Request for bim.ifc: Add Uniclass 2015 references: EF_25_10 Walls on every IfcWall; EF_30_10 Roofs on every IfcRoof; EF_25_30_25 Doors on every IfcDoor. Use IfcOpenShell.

First a look at what the model holds.

```python
import ifcopenshell

model = ifcopenshell.open("bim.ifc")
print(model.schema)
print("classifications:", [c.Name for c in model.by_type("IfcClassification")])
for ifc_class in ("IfcDoor", "IfcRoof", "IfcStair", "IfcWall", "IfcWindow"):
    print(ifc_class, len(model.by_type(ifc_class)))
```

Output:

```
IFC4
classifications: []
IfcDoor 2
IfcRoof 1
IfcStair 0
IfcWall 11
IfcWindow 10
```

```python
import ifcopenshell
import ifcopenshell.api.classification

model = ifcopenshell.open("bim.ifc")

system = ifcopenshell.api.classification.add_classification(model, classification="Uniclass 2015")

codes = {
    "IfcWall": ("EF_25_10", "Walls"),
    "IfcRoof": ("EF_30_10", "Roofs"),
    "IfcDoor": ("EF_25_30_25", "Doors"),
}
for ifc_class, (code, name) in codes.items():
    products = model.by_type(ifc_class)
    ifcopenshell.api.classification.add_reference(
        model, products=products, classification=system, identification=code, name=name
    )
    print(code, len(products))

model.write("bim_updated.ifc")
```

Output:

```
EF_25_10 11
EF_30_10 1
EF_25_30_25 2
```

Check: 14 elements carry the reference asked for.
